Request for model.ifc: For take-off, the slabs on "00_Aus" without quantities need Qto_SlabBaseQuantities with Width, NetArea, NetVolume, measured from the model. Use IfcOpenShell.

First a look at what the model holds.

```python
import ifcopenshell
import ifcopenshell.util.element
import ifcopenshell.util.unit

model = ifcopenshell.open("model.ifc")
print(model.schema)
for unit_type in ("LENGTHUNIT", "AREAUNIT", "VOLUMEUNIT"):
    print(unit_type, ifcopenshell.util.unit.calculate_unit_scale(model, unit_type))
storey = next(s for s in model.by_type("IfcBuildingStorey") if s.Name == "00_Aus")
slabs = [e for e in ifcopenshell.util.element.get_decomposition(storey) if e.is_a("IfcSlab")]
for e in sorted(slabs, key=lambda e: e.id()):
    print(e.id(), e.is_a(), e.Name, list(ifcopenshell.util.element.get_psets(e, qtos_only=True)), sep=" | ")
```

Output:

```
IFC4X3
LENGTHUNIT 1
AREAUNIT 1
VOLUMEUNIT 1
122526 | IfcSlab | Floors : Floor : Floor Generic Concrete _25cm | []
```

```python
import ifcopenshell
import ifcopenshell.api.pset
import ifcopenshell.geom
import ifcopenshell.util.element
import ifcopenshell.util.shape
import ifcopenshell.util.unit

model = ifcopenshell.open("model.ifc")
unit_scale = ifcopenshell.util.unit.calculate_unit_scale(model)
area_scale = ifcopenshell.util.unit.calculate_unit_scale(model, "AREAUNIT")
volume_scale = ifcopenshell.util.unit.calculate_unit_scale(model, "VOLUMEUNIT")
settings = ifcopenshell.geom.settings()

storey = next(s for s in model.by_type("IfcBuildingStorey") if s.Name == "00_Aus")
slabs = [e for e in ifcopenshell.util.element.get_decomposition(storey) if e.is_a("IfcSlab")]

for e in sorted(slabs, key=lambda e: e.id()):
    if ifcopenshell.util.element.get_psets(e, qtos_only=True, should_inherit=False):
        continue
    # Geometry comes back in metres, in the element's own axes.
    shape = ifcopenshell.geom.create_shape(settings, e)
    values = {
        "Width": ifcopenshell.util.shape.get_z(shape.geometry) / unit_scale,
        "NetArea": ifcopenshell.util.shape.get_footprint_area(shape.geometry) / area_scale,
        "NetVolume": ifcopenshell.util.shape.get_volume(shape.geometry) / volume_scale,
    }
    qto = ifcopenshell.api.pset.add_qto(model, product=e, name="Qto_SlabBaseQuantities")
    ifcopenshell.api.pset.edit_qto(model, qto=qto, properties=values)
    print(e.id(), {k: round(v, 3) for k, v in values.items()})

model.write("model_edited.ifc")
```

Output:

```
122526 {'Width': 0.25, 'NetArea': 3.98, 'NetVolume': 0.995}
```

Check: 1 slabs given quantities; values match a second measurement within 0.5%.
